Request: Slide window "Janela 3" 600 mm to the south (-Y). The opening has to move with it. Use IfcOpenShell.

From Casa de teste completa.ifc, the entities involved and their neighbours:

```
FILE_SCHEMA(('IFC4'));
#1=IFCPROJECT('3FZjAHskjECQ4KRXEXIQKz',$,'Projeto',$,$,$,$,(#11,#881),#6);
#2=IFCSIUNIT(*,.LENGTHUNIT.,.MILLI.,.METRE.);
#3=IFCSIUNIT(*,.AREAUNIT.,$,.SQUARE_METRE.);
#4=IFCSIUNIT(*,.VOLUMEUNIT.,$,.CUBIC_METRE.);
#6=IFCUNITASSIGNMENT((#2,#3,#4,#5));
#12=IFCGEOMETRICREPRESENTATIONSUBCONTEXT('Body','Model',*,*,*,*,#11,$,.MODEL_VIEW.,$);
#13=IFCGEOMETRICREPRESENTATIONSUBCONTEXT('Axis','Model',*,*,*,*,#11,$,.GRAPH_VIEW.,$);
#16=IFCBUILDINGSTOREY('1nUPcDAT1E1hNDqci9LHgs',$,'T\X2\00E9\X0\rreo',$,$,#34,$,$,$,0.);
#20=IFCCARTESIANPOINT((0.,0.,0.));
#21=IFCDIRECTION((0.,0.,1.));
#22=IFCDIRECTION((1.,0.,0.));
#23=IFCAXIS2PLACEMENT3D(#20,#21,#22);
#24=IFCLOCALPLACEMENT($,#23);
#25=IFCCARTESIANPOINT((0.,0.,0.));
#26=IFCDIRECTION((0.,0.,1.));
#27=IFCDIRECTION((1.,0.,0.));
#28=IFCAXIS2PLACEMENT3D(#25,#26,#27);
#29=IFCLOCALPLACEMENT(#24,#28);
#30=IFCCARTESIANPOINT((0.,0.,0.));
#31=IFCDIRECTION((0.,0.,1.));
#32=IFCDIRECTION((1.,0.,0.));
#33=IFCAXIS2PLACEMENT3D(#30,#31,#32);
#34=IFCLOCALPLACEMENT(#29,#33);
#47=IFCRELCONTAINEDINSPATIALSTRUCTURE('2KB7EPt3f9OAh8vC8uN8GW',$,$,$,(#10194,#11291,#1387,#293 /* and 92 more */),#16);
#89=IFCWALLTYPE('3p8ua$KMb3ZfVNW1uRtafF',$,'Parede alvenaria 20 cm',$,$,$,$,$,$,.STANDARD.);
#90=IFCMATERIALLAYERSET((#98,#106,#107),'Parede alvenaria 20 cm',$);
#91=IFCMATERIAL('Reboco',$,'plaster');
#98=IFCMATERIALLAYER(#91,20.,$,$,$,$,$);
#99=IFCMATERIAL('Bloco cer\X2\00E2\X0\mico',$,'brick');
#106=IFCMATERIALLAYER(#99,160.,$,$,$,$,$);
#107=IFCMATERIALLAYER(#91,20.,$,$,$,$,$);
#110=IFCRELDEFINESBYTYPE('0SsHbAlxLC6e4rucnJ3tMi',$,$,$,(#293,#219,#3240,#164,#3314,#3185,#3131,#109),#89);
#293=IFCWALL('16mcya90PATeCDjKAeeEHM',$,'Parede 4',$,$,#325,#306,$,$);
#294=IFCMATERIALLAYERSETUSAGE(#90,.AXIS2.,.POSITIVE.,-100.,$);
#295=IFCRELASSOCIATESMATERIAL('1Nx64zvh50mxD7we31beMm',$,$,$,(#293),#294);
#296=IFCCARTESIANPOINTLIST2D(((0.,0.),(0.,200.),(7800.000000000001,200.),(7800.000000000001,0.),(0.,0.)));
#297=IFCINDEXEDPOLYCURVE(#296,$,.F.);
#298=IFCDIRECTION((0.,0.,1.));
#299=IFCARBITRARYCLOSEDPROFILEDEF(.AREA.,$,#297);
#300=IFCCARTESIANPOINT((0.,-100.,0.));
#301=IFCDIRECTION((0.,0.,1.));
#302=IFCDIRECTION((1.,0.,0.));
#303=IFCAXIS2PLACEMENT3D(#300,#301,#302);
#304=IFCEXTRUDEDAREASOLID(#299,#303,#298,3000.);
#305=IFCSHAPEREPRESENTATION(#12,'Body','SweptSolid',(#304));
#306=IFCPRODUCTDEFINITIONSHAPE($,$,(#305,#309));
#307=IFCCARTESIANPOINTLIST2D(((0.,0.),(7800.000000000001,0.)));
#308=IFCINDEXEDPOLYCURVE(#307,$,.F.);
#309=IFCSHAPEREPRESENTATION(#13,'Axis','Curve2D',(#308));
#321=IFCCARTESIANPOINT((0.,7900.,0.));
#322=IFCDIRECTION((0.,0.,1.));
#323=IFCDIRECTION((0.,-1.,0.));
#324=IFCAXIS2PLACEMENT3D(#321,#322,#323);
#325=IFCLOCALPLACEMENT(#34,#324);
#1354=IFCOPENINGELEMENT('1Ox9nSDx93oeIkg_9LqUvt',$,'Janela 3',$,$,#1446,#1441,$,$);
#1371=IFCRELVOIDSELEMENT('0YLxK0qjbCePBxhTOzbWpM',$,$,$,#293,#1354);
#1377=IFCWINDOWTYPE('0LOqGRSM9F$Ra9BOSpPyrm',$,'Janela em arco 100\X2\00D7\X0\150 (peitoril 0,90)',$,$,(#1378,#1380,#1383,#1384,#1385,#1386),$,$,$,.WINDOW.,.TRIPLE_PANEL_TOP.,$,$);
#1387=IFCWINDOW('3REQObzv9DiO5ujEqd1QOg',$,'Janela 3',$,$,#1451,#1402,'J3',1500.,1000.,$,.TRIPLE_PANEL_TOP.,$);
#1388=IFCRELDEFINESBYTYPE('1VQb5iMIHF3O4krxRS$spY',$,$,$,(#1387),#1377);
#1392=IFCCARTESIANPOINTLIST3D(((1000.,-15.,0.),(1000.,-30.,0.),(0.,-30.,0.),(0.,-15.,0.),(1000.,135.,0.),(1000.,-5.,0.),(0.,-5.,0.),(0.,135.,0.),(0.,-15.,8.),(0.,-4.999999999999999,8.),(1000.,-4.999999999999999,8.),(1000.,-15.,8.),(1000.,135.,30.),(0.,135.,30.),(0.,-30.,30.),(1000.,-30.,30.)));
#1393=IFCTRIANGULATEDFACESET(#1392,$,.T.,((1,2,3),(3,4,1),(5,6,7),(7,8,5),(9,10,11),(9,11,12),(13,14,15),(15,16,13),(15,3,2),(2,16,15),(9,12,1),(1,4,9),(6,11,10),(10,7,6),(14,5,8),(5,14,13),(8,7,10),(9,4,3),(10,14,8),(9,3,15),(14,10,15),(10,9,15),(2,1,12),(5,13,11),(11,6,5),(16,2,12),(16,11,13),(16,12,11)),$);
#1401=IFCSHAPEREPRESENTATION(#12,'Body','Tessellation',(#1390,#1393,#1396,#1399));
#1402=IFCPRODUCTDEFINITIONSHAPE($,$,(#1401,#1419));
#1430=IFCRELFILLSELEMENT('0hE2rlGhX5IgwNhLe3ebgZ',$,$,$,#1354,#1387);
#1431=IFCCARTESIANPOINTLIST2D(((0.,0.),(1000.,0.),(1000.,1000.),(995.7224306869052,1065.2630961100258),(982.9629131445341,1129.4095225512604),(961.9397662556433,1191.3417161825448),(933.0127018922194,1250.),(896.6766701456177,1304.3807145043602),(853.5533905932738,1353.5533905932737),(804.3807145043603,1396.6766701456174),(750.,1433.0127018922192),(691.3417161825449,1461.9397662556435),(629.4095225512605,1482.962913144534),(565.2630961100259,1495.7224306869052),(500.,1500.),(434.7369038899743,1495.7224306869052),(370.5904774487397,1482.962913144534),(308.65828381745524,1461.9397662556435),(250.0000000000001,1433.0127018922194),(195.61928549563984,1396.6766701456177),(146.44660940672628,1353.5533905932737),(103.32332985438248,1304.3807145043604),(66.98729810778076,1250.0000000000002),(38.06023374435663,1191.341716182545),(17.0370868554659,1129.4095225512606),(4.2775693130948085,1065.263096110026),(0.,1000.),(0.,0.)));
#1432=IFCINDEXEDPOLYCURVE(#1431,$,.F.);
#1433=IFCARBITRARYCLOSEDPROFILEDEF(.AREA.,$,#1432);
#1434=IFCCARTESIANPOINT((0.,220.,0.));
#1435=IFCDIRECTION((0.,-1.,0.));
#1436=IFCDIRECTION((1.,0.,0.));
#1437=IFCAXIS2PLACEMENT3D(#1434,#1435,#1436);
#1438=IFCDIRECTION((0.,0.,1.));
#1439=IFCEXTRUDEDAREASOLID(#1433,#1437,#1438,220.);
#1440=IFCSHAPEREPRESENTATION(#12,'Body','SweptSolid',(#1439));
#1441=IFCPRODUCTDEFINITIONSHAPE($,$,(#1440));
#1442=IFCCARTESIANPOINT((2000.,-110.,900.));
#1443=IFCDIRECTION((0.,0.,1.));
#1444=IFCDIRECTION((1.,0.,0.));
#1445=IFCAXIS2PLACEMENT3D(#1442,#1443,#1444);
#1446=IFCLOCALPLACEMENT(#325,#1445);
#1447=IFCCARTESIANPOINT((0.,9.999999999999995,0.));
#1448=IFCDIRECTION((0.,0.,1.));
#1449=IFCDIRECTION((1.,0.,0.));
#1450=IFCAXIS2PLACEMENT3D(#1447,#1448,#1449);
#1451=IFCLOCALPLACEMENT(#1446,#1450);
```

```python
import ifcopenshell
import ifcopenshell.api.geometry
import ifcopenshell.util.placement

model = ifcopenshell.open("Casa de teste completa.ifc")

window = model.by_guid("3REQObzv9DiO5ujEqd1QOg")
opening = window.FillsVoids[0].RelatingOpeningElement
wall = opening.VoidsElements[0].RelatingBuildingElement

wall_matrix = ifcopenshell.util.placement.get_local_placement(wall.ObjectPlacement)
shift = wall_matrix[:3, 0] * 600.0
before = ifcopenshell.util.placement.get_local_placement(window.ObjectPlacement)[:3, 3].copy()

# The window is placed relative to its opening, so it follows when the opening moves.
matrix = ifcopenshell.util.placement.get_local_placement(opening.ObjectPlacement)
matrix[:3, 3] += shift
ifcopenshell.api.geometry.edit_object_placement(
    model, product=opening, matrix=matrix, is_si=False, should_transform_children=True
)

after = ifcopenshell.util.placement.get_local_placement(window.ObjectPlacement)[:3, 3]
print("window moved by", (after - before).round(3) + 0.0)

model.write("Casa de teste completa-out.ifc")
```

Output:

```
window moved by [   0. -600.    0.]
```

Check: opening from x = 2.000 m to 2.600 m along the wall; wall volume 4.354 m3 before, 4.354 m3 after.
